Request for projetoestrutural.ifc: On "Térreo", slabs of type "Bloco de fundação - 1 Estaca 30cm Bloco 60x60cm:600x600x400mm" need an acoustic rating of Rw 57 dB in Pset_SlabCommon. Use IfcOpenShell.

First a look at what the model holds.

```python
import ifcopenshell
import ifcopenshell.util.element

model = ifcopenshell.open("projetoestrutural.ifc")
print(model.schema)
storey = next(s for s in model.by_type("IfcBuildingStorey") if s.Name == "Térreo")
slabs = [e for e in ifcopenshell.util.element.get_decomposition(storey) if e.is_a("IfcSlab")]
seen = {}
for e in slabs:
    element_type = ifcopenshell.util.element.get_type(e)
    key = (element_type.Name if element_type != e and element_type else None, ifcopenshell.util.element.get_pset(e, "Pset_SlabCommon", "AcousticRating"))
    seen[key] = seen.get(key, 0) + 1
for (name, value), count in sorted(seen.items(), key=str):
    print(count, "x", name, "|", value)
```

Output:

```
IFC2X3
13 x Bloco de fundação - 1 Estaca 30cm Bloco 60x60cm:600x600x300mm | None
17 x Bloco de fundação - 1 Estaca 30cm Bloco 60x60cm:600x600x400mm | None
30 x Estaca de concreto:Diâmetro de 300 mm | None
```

```python
import ifcopenshell
import ifcopenshell.api.pset
import ifcopenshell.util.element

model = ifcopenshell.open("projetoestrutural.ifc")

storey = next(s for s in model.by_type("IfcBuildingStorey") if s.Name == "Térreo")
slabs = [e for e in ifcopenshell.util.element.get_decomposition(storey) if e.is_a("IfcSlab")]

count = 0
for e in slabs:
    element_type = ifcopenshell.util.element.get_type(e)
    if element_type in (None, e) or element_type.Name != "Bloco de fundação - 1 Estaca 30cm Bloco 60x60cm:600x600x400mm":
        continue
    # add_pset returns the element's existing set when there is one.
    pset = ifcopenshell.api.pset.add_pset(model, product=e, name="Pset_SlabCommon")
    ifcopenshell.api.pset.edit_pset(model, pset=pset, properties={"AcousticRating": "Rw 57 dB"})
    count += 1

print(count, "slabs updated")

model.write("projetoestrutural_edited.ifc")
```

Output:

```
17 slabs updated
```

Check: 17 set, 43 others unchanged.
